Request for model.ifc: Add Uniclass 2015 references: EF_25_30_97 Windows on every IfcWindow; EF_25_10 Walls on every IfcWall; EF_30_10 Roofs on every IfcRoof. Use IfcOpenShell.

First a look at what the model holds.

```python
import ifcopenshell

model = ifcopenshell.open("model.ifc")
print(model.schema)
print("classifications:", [c.Name for c in model.by_type("IfcClassification")])
for ifc_class in ("IfcDoor", "IfcRoof", "IfcStair", "IfcWall", "IfcWindow"):
    print(ifc_class, len(model.by_type(ifc_class)))
```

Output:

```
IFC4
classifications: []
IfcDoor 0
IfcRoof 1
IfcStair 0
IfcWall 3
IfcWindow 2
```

```python
import ifcopenshell
import ifcopenshell.api.classification

model = ifcopenshell.open("model.ifc")

system = ifcopenshell.api.classification.add_classification(model, classification="Uniclass 2015")

codes = {
    "IfcWindow": ("EF_25_30_97", "Windows"),
    "IfcWall": ("EF_25_10", "Walls"),
    "IfcRoof": ("EF_30_10", "Roofs"),
}
for ifc_class, (code, name) in codes.items():
    products = model.by_type(ifc_class)
    ifcopenshell.api.classification.add_reference(
        model, products=products, classification=system, identification=code, name=name
    )
    print(code, len(products))

model.write("model_updated.ifc")
```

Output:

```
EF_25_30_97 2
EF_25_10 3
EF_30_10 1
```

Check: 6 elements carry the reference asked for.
